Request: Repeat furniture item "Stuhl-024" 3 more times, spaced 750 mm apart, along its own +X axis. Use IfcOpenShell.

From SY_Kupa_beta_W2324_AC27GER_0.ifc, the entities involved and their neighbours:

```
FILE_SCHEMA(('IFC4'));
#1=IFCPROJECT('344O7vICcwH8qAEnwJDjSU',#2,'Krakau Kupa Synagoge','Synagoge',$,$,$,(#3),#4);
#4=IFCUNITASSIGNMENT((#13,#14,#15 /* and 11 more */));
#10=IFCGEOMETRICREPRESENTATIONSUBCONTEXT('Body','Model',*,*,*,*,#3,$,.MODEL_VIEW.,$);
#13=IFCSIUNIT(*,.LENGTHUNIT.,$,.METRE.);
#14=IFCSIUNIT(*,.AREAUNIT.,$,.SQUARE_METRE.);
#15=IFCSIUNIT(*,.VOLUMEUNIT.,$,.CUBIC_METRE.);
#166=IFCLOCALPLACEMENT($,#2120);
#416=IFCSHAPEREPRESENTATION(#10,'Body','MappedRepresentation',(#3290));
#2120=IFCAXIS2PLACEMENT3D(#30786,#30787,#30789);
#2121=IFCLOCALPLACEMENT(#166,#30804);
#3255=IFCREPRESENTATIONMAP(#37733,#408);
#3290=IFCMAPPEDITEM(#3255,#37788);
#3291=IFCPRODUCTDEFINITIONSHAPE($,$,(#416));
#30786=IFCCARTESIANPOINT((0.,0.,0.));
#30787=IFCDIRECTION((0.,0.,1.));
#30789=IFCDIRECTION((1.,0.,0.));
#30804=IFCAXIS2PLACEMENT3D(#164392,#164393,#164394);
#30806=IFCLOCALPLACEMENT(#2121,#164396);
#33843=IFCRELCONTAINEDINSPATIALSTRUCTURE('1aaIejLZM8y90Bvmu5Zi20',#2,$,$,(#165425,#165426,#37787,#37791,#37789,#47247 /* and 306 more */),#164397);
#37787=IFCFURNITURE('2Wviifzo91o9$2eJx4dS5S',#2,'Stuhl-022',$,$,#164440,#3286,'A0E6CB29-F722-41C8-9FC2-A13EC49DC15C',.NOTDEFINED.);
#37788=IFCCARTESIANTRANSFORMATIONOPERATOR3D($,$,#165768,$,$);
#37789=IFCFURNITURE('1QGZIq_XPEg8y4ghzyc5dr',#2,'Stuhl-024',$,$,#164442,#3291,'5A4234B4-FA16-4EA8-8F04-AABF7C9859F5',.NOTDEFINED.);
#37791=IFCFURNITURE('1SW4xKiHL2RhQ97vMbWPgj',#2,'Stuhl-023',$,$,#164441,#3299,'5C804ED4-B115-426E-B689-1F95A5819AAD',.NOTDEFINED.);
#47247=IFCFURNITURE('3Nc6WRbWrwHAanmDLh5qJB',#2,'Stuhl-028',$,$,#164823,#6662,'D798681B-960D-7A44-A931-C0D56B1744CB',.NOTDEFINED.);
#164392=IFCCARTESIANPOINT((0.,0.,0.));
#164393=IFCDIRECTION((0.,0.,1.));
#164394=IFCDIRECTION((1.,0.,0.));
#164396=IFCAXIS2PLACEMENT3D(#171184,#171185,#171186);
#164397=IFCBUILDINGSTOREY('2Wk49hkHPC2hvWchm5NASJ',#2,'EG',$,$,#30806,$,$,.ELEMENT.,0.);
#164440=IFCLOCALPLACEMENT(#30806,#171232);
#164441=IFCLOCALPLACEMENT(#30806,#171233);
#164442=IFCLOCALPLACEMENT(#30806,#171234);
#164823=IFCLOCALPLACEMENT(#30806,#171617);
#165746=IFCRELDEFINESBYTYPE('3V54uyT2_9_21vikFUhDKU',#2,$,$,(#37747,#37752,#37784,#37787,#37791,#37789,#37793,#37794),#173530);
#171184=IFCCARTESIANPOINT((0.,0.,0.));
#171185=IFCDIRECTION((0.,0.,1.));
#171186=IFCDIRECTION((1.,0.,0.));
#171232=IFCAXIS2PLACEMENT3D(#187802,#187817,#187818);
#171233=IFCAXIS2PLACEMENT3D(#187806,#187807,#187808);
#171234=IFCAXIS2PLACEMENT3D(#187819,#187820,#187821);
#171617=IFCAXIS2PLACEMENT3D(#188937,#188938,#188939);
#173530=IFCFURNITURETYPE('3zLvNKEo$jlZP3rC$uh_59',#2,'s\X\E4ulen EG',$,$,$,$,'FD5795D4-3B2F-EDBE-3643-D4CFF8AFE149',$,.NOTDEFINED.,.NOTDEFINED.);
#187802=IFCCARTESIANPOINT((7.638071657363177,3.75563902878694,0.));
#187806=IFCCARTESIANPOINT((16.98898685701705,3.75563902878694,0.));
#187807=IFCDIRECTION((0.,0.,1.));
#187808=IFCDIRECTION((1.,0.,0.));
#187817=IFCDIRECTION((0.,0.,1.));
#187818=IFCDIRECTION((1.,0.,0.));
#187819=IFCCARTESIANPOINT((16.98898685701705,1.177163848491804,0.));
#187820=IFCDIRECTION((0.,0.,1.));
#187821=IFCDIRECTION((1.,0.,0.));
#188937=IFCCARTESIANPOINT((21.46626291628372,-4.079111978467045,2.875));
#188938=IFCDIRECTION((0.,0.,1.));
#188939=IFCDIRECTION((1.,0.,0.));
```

```python
import ifcopenshell
import ifcopenshell.api.geometry
import ifcopenshell.api.root
import ifcopenshell.util.element
import ifcopenshell.util.placement
import ifcopenshell.util.unit

model = ifcopenshell.open("SY_Kupa_beta_W2324_AC27GER_0.ifc")
unit_scale = ifcopenshell.util.unit.calculate_unit_scale(model)


def reuse_history(source, copy):
    """copy_class also copies each property set's owner history, people and application; keep the originals."""
    for rel in copy.IsDefinedBy:
        if rel.is_a("IfcRelDefinesByProperties") and (history := rel.RelatingPropertyDefinition.OwnerHistory):
            rel.RelatingPropertyDefinition.OwnerHistory = source.OwnerHistory
            ifcopenshell.util.element.remove_deep2(model, history)


source = model.by_guid("1QGZIq_XPEg8y4ghzyc5dr")
base = ifcopenshell.util.placement.get_local_placement(source.ObjectPlacement)
step = base[:3, 0] * 0.75 / unit_scale

for i in range(1, 4):
    copy = ifcopenshell.api.root.copy_class(model, product=source)
    copy.Representation = ifcopenshell.util.element.copy_deep(
        model, source.Representation, exclude=["IfcGeometricRepresentationContext", "IfcRepresentationMap"]
    )
    copy.Tag = None
    reuse_history(source, copy)
    matrix = base.copy()
    matrix[:3, 3] += i * step
    print("added at", matrix[:3, 3].round(3) + 0.0)
    ifcopenshell.api.geometry.edit_object_placement(model, product=copy, matrix=matrix, is_si=False)

model.write("SY_Kupa_beta_W2324_AC27GER_0-out.ifc")
```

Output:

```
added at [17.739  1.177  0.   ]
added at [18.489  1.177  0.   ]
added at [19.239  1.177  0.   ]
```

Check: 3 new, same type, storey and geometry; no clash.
